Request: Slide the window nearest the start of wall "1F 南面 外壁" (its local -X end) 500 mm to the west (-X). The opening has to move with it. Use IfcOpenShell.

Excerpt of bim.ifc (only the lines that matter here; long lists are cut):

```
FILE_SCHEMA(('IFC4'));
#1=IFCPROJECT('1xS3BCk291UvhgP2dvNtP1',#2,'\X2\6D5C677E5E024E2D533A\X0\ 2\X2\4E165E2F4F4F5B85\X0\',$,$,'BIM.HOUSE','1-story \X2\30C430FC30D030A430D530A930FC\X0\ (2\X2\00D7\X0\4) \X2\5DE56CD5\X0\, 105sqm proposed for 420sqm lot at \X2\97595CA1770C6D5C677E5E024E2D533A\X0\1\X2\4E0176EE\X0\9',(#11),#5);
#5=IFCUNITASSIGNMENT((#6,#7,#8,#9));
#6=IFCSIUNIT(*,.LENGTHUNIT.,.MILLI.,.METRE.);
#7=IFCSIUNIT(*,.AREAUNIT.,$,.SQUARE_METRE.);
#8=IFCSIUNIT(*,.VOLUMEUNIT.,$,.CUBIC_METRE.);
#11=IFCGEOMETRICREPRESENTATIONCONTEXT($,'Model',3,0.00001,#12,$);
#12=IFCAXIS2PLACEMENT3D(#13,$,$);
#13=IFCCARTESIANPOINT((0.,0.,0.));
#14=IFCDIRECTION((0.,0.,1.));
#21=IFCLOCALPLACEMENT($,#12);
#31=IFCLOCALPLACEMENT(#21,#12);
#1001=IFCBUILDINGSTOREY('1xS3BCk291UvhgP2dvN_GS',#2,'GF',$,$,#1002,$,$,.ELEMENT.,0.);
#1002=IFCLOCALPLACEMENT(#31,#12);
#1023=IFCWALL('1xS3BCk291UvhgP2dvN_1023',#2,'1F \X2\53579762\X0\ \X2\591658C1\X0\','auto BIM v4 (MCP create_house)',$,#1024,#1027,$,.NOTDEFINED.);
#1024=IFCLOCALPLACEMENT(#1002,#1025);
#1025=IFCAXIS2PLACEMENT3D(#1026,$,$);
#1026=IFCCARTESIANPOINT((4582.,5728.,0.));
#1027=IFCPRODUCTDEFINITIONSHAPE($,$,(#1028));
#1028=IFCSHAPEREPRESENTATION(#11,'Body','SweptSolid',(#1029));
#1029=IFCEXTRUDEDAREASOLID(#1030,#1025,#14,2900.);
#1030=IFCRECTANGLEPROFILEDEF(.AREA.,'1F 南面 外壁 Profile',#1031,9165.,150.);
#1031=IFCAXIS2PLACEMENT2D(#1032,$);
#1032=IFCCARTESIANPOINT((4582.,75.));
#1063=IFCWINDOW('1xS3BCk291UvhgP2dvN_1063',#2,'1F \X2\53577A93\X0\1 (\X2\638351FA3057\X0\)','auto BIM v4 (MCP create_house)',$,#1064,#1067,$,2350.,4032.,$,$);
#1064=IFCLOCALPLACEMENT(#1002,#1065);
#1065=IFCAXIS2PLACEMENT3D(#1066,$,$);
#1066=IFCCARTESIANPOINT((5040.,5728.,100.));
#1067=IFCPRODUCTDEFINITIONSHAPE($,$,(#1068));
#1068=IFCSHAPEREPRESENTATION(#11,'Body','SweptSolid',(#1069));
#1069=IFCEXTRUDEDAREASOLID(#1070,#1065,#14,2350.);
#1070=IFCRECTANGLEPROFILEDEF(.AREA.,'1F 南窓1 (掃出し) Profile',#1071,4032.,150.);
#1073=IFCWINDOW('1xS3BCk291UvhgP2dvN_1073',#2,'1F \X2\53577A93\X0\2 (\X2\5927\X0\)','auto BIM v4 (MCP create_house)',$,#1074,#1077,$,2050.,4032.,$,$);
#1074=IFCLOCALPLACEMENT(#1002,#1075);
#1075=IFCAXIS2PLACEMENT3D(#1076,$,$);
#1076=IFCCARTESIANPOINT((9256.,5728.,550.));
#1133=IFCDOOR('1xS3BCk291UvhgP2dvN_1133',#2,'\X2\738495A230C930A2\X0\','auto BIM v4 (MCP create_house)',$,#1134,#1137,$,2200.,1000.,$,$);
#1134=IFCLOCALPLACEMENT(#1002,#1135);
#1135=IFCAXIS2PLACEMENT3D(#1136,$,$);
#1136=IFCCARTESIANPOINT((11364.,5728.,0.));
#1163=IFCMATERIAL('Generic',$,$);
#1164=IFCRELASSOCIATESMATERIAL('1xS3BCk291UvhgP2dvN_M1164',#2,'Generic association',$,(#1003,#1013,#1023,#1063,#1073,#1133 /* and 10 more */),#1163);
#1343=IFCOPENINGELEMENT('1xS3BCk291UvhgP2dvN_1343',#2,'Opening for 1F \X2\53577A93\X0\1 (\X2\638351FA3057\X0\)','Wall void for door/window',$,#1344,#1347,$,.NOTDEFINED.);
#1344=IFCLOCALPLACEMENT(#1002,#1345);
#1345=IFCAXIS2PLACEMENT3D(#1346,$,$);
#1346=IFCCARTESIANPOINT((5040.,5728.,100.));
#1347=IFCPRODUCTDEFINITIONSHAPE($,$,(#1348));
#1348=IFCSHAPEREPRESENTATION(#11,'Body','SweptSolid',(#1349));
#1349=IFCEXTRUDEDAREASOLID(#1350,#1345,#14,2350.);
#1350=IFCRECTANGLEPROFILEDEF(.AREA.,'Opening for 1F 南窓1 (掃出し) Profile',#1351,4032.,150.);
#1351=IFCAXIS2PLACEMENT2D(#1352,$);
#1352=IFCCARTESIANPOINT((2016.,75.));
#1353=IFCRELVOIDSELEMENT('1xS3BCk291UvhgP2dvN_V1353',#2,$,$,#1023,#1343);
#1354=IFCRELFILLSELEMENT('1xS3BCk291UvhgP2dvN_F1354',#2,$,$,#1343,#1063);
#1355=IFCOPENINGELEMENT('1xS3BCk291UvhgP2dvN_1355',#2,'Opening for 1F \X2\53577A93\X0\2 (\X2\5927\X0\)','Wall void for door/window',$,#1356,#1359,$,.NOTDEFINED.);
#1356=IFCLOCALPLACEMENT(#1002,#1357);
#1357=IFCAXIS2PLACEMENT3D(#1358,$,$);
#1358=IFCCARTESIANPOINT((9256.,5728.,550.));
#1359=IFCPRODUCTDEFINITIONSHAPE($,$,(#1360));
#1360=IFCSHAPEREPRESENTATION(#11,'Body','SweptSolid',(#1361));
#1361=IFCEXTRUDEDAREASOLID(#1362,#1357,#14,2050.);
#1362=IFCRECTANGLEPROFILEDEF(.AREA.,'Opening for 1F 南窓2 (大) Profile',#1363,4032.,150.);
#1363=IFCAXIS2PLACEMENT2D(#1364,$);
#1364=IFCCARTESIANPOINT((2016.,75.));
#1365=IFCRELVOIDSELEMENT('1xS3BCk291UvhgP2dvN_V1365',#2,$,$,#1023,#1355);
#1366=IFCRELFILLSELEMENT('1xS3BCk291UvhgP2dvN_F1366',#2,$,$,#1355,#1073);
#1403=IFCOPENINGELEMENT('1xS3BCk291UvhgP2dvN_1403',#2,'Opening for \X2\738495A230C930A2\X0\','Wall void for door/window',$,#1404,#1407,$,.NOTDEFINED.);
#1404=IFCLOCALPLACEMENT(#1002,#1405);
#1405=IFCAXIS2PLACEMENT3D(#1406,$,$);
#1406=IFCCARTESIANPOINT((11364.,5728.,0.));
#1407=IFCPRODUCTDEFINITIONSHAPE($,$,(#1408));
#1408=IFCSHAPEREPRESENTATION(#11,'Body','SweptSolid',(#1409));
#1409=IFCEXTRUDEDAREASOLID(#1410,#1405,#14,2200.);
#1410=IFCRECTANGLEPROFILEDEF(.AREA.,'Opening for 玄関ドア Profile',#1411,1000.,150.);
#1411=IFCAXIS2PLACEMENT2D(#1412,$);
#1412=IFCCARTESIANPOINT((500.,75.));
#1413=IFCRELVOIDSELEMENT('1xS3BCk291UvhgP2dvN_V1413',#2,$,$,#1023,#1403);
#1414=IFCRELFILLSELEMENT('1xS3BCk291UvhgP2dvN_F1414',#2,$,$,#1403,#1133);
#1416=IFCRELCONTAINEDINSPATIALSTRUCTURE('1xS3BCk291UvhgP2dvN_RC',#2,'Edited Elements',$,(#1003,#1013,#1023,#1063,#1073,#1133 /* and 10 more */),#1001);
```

```python
import ifcopenshell
import ifcopenshell.api.geometry
import ifcopenshell.util.placement
import ifcopenshell.util.unit

model = ifcopenshell.open("bim.ifc")
unit_scale = ifcopenshell.util.unit.calculate_unit_scale(model)

window = model.by_guid("1xS3BCk291UvhgP2dvN_1063")
opening = window.FillsVoids[0].RelatingOpeningElement
wall = opening.VoidsElements[0].RelatingBuildingElement

wall_matrix = ifcopenshell.util.placement.get_local_placement(wall.ObjectPlacement)
shift = wall_matrix[:3, 0] * -0.5 / unit_scale
before = ifcopenshell.util.placement.get_local_placement(window.ObjectPlacement)[:3, 3].copy()

# The window is not placed relative to its opening, so move both.
for product in (opening, window):
    matrix = ifcopenshell.util.placement.get_local_placement(product.ObjectPlacement)
    matrix[:3, 3] += shift
    ifcopenshell.api.geometry.edit_object_placement(model, product=product, matrix=matrix, is_si=False)

after = ifcopenshell.util.placement.get_local_placement(window.ObjectPlacement)[:3, 3]
print("window moved by", (after - before).round(3) + 0.0)

model.write("bim_v2.ifc")
```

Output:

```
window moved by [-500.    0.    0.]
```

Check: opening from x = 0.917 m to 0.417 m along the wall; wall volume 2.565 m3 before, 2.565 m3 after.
